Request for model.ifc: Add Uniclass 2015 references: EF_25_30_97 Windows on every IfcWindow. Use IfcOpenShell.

First a look at what the model holds.

```python
import ifcopenshell

model = ifcopenshell.open("model.ifc")
print(model.schema)
print("classifications:", [c.Name for c in model.by_type("IfcClassification")])
for ifc_class in ("IfcDoor", "IfcRoof", "IfcStair", "IfcWall", "IfcWindow"):
    print(ifc_class, len(model.by_type(ifc_class)))
```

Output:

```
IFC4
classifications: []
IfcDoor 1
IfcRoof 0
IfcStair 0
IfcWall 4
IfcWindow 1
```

```python
import ifcopenshell
import ifcopenshell.api.classification

model = ifcopenshell.open("model.ifc")

system = ifcopenshell.api.classification.add_classification(model, classification="Uniclass 2015")

codes = {
    "IfcWindow": ("EF_25_30_97", "Windows"),
}
for ifc_class, (code, name) in codes.items():
    products = model.by_type(ifc_class)
    ifcopenshell.api.classification.add_reference(
        model, products=products, classification=system, identification=code, name=name
    )
    print(code, len(products))

model.write("model_v2.ifc")
```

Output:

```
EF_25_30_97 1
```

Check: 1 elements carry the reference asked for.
